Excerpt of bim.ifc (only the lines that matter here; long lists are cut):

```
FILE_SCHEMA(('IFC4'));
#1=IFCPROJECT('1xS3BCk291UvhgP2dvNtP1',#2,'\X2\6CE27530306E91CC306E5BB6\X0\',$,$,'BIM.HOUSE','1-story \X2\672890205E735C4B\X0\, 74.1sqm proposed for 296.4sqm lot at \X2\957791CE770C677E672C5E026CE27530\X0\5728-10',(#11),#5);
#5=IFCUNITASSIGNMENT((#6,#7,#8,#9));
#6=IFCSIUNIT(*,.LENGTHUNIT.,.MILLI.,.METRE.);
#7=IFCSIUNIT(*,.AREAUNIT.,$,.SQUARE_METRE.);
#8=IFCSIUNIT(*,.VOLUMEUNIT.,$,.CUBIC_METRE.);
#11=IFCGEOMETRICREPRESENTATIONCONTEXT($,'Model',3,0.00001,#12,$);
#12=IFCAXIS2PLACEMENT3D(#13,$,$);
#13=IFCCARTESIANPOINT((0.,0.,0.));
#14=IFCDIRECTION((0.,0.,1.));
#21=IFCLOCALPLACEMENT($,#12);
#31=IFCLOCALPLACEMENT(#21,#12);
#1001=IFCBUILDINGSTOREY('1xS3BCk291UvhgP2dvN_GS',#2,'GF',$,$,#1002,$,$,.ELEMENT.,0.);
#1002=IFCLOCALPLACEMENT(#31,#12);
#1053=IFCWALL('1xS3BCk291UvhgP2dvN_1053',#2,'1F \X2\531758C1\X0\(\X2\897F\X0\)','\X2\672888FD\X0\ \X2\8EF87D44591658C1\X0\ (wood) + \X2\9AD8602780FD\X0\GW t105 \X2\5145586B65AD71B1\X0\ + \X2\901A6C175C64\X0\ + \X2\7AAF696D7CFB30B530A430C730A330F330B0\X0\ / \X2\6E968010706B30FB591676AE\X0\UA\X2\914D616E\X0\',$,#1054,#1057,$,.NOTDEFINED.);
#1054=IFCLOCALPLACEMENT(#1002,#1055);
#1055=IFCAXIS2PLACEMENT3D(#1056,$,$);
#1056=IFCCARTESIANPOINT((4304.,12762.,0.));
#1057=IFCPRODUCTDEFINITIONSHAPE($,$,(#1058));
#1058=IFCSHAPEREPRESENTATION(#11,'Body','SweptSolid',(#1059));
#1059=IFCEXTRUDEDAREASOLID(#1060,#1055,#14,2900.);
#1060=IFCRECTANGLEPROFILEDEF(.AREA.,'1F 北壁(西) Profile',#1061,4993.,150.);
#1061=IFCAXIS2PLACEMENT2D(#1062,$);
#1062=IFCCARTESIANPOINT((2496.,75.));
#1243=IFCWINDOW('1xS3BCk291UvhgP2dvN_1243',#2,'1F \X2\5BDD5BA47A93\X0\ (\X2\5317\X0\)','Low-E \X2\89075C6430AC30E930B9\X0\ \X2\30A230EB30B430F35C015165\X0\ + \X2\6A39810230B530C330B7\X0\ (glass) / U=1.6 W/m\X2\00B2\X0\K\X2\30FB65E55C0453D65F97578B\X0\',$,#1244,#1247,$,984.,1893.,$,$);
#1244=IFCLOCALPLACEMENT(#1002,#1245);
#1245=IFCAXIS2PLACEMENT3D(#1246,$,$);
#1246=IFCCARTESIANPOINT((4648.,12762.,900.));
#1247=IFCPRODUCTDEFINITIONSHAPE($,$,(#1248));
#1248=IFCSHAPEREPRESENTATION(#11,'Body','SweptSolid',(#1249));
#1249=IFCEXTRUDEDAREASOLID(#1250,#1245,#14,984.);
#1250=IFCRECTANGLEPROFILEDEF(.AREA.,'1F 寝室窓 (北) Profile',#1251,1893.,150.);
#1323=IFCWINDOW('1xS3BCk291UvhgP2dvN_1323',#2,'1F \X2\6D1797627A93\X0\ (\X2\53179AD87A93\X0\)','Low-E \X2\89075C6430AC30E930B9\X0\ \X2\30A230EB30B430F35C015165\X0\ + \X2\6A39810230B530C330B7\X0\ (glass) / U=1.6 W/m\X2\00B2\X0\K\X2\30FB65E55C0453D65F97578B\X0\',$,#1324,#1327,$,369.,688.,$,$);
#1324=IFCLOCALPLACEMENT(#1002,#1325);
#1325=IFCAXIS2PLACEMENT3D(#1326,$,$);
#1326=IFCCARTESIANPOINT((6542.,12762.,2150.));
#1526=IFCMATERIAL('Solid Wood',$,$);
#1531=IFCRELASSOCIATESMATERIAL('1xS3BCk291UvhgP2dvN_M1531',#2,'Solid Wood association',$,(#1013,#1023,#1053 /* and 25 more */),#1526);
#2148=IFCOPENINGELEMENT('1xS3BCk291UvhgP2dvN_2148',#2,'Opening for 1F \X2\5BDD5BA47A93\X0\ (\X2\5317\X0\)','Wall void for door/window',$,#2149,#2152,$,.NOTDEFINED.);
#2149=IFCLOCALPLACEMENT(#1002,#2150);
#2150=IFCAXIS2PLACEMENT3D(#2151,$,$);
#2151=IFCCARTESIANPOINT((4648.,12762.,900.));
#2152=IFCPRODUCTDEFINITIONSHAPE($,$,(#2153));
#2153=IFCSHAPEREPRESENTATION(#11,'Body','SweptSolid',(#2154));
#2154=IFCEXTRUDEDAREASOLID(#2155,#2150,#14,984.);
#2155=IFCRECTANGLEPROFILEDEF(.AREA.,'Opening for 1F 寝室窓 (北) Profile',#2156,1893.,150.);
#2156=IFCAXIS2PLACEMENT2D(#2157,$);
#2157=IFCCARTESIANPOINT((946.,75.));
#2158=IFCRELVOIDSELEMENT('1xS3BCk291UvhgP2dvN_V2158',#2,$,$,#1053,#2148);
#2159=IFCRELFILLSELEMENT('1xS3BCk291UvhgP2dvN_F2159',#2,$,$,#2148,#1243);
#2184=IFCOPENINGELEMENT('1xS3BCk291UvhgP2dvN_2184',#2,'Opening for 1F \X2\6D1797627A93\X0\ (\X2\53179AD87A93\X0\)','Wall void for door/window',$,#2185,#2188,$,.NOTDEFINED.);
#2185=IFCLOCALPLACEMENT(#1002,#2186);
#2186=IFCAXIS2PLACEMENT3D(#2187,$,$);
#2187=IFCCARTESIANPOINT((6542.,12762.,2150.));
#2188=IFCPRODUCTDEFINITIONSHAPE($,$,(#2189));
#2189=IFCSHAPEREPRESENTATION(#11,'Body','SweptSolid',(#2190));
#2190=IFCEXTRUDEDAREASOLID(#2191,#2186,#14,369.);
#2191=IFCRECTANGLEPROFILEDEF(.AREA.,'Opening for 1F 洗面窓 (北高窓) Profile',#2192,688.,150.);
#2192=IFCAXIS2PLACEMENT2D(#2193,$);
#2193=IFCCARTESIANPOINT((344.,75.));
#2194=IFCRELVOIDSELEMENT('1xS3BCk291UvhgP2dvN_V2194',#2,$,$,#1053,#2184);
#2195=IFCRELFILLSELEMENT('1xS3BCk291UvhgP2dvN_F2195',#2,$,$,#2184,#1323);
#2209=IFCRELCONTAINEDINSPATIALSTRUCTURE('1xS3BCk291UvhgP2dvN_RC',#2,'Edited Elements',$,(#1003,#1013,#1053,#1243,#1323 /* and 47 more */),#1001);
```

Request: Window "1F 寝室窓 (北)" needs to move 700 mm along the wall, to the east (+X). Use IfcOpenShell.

```python
import ifcopenshell
import ifcopenshell.api.geometry
import ifcopenshell.util.placement

model = ifcopenshell.open("bim.ifc")

window = model.by_guid("1xS3BCk291UvhgP2dvN_1243")
opening = window.FillsVoids[0].RelatingOpeningElement
wall = opening.VoidsElements[0].RelatingBuildingElement

wall_matrix = ifcopenshell.util.placement.get_local_placement(wall.ObjectPlacement)
shift = wall_matrix[:3, 0] * 700.0
before = ifcopenshell.util.placement.get_local_placement(window.ObjectPlacement)[:3, 3].copy()

# The window is not placed relative to its opening, so move both.
for product in (opening, window):
    matrix = ifcopenshell.util.placement.get_local_placement(product.ObjectPlacement)
    matrix[:3, 3] += shift
    ifcopenshell.api.geometry.edit_object_placement(model, product=product, matrix=matrix, is_si=False)

after = ifcopenshell.util.placement.get_local_placement(window.ObjectPlacement)[:3, 3]
print("window moved by", (after - before).round(3) + 0.0)

model.write("bim_edited.ifc")
```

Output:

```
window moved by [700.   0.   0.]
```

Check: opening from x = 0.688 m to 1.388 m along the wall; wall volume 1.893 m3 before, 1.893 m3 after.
